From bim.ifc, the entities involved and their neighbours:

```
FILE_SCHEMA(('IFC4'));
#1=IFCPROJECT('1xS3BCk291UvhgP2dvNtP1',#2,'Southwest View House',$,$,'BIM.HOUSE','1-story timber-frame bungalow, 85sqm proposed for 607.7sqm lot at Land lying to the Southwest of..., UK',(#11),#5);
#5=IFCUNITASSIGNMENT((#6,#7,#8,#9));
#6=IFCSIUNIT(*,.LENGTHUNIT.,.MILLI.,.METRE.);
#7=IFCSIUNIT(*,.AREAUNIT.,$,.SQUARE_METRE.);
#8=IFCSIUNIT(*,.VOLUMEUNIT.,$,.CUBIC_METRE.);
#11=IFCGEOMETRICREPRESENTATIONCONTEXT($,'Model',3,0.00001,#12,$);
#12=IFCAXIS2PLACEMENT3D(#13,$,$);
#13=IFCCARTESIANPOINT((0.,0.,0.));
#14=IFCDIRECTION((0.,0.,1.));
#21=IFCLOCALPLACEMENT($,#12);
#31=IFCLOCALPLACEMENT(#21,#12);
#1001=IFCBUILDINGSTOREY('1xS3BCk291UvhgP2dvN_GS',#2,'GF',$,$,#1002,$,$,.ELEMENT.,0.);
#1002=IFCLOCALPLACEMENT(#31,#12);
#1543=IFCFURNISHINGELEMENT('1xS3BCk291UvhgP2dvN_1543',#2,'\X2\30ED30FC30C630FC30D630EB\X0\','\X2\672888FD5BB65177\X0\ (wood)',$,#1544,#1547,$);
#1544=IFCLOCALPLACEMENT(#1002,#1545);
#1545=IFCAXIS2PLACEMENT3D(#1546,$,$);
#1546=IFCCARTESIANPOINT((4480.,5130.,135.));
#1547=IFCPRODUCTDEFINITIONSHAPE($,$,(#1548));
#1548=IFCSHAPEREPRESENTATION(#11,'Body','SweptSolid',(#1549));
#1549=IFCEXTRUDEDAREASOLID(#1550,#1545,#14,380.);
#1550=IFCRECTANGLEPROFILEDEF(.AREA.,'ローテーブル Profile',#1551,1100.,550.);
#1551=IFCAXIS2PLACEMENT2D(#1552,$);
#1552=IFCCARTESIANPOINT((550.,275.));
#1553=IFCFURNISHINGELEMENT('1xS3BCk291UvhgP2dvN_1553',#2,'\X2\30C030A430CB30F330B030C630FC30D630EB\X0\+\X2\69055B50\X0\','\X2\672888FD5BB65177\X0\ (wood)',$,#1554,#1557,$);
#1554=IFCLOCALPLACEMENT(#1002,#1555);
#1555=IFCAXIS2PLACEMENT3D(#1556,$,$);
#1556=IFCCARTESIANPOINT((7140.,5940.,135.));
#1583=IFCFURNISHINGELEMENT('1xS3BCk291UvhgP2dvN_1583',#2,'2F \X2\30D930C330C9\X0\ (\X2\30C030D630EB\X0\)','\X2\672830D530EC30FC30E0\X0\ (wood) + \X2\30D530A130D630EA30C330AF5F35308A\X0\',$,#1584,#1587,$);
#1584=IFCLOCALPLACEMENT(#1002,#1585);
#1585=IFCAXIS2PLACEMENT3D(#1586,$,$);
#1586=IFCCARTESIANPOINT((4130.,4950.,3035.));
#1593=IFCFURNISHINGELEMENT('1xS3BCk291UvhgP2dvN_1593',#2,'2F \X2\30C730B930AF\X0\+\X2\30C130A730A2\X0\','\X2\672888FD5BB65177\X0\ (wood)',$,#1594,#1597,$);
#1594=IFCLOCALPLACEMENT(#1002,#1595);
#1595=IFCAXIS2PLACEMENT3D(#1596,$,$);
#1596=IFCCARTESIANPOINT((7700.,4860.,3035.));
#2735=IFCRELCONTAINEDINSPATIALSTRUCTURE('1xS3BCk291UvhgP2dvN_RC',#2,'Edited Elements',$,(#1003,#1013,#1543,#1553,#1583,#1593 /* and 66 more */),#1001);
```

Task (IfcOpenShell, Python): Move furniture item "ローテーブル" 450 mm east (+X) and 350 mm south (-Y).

```python
import ifcopenshell
import ifcopenshell.api.geometry
import ifcopenshell.util.placement

model = ifcopenshell.open("bim.ifc")

item = model.by_guid("1xS3BCk291UvhgP2dvN_1543")
matrix = ifcopenshell.util.placement.get_local_placement(item.ObjectPlacement)
matrix[0, 3] += 450.0
matrix[1, 3] -= 350.0
ifcopenshell.api.geometry.edit_object_placement(model, product=item, matrix=matrix, is_si=False)

print(ifcopenshell.util.placement.get_local_placement(item.ObjectPlacement).round(3) + 0.0)

model.write("bim_updated.ifc")
```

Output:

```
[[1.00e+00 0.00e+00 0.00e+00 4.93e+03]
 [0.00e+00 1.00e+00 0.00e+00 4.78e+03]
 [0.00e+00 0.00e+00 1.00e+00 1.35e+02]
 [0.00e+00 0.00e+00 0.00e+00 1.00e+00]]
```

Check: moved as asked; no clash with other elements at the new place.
